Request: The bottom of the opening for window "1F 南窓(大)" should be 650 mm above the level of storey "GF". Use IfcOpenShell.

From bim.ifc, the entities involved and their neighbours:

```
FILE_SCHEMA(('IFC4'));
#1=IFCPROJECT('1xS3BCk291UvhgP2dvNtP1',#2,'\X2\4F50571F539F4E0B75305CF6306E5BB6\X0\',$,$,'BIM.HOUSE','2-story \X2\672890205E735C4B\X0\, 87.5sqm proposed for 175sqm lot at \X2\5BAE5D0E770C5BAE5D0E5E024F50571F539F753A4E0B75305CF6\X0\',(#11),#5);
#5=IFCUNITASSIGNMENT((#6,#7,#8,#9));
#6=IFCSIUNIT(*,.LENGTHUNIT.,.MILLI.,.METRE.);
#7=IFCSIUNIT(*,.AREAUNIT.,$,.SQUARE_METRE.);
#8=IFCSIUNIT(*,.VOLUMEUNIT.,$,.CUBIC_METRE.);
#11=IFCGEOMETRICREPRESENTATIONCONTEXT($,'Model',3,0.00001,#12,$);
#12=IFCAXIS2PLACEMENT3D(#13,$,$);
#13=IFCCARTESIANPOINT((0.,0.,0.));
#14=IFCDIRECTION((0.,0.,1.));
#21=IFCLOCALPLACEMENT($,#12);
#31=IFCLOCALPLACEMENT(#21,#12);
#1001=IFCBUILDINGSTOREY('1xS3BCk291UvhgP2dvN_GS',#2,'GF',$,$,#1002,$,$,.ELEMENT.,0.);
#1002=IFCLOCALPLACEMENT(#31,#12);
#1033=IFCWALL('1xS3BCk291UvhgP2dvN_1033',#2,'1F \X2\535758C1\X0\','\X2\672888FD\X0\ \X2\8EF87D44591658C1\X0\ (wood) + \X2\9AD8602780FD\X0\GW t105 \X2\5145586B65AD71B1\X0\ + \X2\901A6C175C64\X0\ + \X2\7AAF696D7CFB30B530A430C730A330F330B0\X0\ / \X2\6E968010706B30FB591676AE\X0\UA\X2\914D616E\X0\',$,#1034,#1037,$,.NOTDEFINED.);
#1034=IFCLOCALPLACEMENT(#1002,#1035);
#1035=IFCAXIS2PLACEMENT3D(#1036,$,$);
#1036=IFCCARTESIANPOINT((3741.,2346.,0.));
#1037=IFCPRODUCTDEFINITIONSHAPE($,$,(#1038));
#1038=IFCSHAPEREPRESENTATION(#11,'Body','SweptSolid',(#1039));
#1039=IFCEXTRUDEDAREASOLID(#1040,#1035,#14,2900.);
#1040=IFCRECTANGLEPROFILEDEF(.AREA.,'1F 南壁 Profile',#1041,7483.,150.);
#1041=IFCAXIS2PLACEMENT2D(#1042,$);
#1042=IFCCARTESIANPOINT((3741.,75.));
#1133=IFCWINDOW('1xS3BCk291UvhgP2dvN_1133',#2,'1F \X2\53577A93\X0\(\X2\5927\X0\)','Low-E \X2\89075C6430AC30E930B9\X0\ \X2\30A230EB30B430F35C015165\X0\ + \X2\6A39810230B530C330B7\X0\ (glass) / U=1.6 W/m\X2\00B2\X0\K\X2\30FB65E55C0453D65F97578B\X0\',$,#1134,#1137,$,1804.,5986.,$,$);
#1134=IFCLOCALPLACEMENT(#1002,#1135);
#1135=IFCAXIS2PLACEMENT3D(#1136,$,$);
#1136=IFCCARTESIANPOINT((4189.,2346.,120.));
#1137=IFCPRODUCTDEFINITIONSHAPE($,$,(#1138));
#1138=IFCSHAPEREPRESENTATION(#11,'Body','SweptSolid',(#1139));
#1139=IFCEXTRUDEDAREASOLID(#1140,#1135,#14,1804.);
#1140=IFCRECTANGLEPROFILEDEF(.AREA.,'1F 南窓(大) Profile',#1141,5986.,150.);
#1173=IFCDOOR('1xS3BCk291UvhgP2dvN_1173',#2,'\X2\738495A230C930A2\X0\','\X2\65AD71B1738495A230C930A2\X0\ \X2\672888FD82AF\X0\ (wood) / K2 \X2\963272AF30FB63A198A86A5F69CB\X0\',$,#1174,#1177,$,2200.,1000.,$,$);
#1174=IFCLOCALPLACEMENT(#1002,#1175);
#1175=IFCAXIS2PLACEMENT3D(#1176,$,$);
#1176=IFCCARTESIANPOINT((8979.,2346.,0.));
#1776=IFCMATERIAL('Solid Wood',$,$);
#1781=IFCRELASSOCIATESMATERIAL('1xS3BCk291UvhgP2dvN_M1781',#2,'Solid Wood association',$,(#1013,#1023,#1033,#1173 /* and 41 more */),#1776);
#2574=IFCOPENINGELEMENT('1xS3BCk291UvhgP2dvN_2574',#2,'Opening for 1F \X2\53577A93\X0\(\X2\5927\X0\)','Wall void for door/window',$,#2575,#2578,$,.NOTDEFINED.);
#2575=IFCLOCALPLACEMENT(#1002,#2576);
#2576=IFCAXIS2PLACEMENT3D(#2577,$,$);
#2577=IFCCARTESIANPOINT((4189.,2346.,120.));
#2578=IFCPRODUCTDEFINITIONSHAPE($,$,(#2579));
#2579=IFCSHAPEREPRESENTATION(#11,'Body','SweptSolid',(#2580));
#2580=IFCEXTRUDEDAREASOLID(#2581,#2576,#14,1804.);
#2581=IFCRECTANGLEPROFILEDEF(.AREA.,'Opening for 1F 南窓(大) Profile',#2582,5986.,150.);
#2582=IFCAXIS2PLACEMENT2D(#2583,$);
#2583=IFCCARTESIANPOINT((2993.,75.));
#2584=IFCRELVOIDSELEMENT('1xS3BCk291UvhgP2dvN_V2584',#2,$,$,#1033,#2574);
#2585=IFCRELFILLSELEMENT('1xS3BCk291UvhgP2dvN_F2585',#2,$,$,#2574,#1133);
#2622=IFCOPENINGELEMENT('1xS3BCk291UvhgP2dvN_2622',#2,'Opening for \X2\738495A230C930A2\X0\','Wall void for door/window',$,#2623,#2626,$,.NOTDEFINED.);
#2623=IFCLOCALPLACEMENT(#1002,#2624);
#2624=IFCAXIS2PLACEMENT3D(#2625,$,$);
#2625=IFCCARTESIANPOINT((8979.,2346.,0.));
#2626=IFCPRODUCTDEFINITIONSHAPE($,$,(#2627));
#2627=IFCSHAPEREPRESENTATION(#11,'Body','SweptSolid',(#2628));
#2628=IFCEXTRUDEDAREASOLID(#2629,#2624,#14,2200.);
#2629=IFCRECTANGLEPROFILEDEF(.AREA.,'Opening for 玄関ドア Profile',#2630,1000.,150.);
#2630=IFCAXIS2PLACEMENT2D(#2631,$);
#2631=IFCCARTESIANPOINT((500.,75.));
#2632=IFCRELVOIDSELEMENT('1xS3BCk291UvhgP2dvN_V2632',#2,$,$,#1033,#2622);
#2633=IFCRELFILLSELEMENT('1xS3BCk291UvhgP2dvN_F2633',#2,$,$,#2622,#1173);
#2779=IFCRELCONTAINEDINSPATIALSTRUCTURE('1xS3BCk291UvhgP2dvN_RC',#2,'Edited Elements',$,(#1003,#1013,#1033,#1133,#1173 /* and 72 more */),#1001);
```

```python
import numpy as np
import ifcopenshell
import ifcopenshell.api.geometry
import ifcopenshell.geom
import ifcopenshell.util.element
import ifcopenshell.util.placement
import ifcopenshell.util.shape
import ifcopenshell.util.unit

model = ifcopenshell.open("bim.ifc")
unit_scale = ifcopenshell.util.unit.calculate_unit_scale(model)

window = model.by_guid("1xS3BCk291UvhgP2dvN_1133")
opening = window.FillsVoids[0].RelatingOpeningElement
storey = ifcopenshell.util.element.get_container(window, ifc_class="IfcBuildingStorey")
level = ifcopenshell.util.placement.get_local_placement(storey.ObjectPlacement)[2, 3]

# The opening's origin need not be at the sill, so measure its lowest point.
shape = ifcopenshell.geom.create_shape(ifcopenshell.geom.settings(), opening)
bottom = ifcopenshell.util.shape.get_shape_bottom_elevation(shape, shape.geometry) / unit_scale
dz = level + 0.65 / unit_scale - bottom

shift = np.array([0.0, 0.0, dz])
# The window is not placed relative to its opening, so move both.
for product in (opening, window):
    matrix = ifcopenshell.util.placement.get_local_placement(product.ObjectPlacement)
    matrix[:3, 3] += shift
    ifcopenshell.api.geometry.edit_object_placement(model, product=product, matrix=matrix, is_si=False)

print(f"moved by {dz * unit_scale:+.3f} m")

model.write("bim_rev.ifc")
```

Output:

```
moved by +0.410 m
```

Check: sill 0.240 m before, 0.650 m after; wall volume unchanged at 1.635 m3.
